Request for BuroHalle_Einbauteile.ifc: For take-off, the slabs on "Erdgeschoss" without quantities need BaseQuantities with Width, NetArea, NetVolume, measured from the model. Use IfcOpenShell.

First a look at what the model holds.

```python
import ifcopenshell
import ifcopenshell.util.element
import ifcopenshell.util.unit

model = ifcopenshell.open("BuroHalle_Einbauteile.ifc")
print(model.schema)
for unit_type in ("LENGTHUNIT", "AREAUNIT", "VOLUMEUNIT"):
    print(unit_type, ifcopenshell.util.unit.calculate_unit_scale(model, unit_type))
storey = next(s for s in model.by_type("IfcBuildingStorey") if s.Name == "Erdgeschoss")
slabs = [e for e in ifcopenshell.util.element.get_decomposition(storey) if e.is_a("IfcSlab")]
for e in sorted(slabs, key=lambda e: e.id()):
    print(e.id(), e.is_a(), e.Name, list(ifcopenshell.util.element.get_psets(e, qtos_only=True)), sep=" | ")
```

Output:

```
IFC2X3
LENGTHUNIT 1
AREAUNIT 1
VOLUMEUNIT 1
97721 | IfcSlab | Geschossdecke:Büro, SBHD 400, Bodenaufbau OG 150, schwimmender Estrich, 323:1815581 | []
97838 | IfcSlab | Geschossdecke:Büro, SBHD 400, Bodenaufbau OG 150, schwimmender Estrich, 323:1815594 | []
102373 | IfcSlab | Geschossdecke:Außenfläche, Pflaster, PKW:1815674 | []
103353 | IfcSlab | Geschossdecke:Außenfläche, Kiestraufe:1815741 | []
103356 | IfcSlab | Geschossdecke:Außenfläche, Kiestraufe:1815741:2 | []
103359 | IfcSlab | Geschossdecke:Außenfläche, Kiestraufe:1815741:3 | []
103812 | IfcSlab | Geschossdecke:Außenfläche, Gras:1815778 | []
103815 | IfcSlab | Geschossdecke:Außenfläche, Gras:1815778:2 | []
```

```python
import ifcopenshell
import ifcopenshell.api.pset
import ifcopenshell.geom
import ifcopenshell.util.element
import ifcopenshell.util.shape
import ifcopenshell.util.unit

model = ifcopenshell.open("BuroHalle_Einbauteile.ifc")
unit_scale = ifcopenshell.util.unit.calculate_unit_scale(model)
area_scale = ifcopenshell.util.unit.calculate_unit_scale(model, "AREAUNIT")
volume_scale = ifcopenshell.util.unit.calculate_unit_scale(model, "VOLUMEUNIT")
settings = ifcopenshell.geom.settings()

storey = next(s for s in model.by_type("IfcBuildingStorey") if s.Name == "Erdgeschoss")
slabs = [e for e in ifcopenshell.util.element.get_decomposition(storey) if e.is_a("IfcSlab")]

for e in sorted(slabs, key=lambda e: e.id()):
    if ifcopenshell.util.element.get_psets(e, qtos_only=True, should_inherit=False):
        continue
    # Geometry comes back in metres, in the element's own axes.
    shape = ifcopenshell.geom.create_shape(settings, e)
    values = {
        "Width": ifcopenshell.util.shape.get_z(shape.geometry) / unit_scale,
        "NetArea": ifcopenshell.util.shape.get_footprint_area(shape.geometry) / area_scale,
        "NetVolume": ifcopenshell.util.shape.get_volume(shape.geometry) / volume_scale,
    }
    qto = ifcopenshell.api.pset.add_qto(model, product=e, name="BaseQuantities")
    ifcopenshell.api.pset.edit_qto(model, qto=qto, properties=values)
    print(e.id(), {k: round(v, 3) for k, v in values.items()})

model.write("BuroHalle_Einbauteile_updated.ifc")
```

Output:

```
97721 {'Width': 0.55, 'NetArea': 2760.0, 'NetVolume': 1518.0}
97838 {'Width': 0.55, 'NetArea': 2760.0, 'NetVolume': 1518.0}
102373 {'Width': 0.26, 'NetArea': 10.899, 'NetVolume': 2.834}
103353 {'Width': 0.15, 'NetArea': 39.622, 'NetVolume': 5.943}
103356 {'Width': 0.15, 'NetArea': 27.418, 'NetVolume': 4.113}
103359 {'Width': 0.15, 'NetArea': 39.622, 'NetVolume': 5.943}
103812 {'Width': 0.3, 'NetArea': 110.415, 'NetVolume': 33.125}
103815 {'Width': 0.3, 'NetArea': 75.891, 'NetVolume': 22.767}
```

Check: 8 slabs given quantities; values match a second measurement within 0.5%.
